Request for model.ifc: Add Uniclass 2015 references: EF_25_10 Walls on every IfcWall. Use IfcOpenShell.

First a look at what the model holds.

```python
import ifcopenshell

model = ifcopenshell.open("model.ifc")
print(model.schema)
print("classifications:", [c.Name for c in model.by_type("IfcClassification")])
for ifc_class in ("IfcDoor", "IfcRoof", "IfcStair", "IfcWall", "IfcWindow"):
    print(ifc_class, len(model.by_type(ifc_class)))
```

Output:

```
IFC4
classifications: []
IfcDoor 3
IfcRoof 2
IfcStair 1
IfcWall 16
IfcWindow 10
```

```python
import ifcopenshell
import ifcopenshell.api.classification

model = ifcopenshell.open("model.ifc")

system = ifcopenshell.api.classification.add_classification(model, classification="Uniclass 2015")

codes = {
    "IfcWall": ("EF_25_10", "Walls"),
}
for ifc_class, (code, name) in codes.items():
    products = model.by_type(ifc_class)
    ifcopenshell.api.classification.add_reference(
        model, products=products, classification=system, identification=code, name=name
    )
    print(code, len(products))

model.write("model_updated.ifc")
```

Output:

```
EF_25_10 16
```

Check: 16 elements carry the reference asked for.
